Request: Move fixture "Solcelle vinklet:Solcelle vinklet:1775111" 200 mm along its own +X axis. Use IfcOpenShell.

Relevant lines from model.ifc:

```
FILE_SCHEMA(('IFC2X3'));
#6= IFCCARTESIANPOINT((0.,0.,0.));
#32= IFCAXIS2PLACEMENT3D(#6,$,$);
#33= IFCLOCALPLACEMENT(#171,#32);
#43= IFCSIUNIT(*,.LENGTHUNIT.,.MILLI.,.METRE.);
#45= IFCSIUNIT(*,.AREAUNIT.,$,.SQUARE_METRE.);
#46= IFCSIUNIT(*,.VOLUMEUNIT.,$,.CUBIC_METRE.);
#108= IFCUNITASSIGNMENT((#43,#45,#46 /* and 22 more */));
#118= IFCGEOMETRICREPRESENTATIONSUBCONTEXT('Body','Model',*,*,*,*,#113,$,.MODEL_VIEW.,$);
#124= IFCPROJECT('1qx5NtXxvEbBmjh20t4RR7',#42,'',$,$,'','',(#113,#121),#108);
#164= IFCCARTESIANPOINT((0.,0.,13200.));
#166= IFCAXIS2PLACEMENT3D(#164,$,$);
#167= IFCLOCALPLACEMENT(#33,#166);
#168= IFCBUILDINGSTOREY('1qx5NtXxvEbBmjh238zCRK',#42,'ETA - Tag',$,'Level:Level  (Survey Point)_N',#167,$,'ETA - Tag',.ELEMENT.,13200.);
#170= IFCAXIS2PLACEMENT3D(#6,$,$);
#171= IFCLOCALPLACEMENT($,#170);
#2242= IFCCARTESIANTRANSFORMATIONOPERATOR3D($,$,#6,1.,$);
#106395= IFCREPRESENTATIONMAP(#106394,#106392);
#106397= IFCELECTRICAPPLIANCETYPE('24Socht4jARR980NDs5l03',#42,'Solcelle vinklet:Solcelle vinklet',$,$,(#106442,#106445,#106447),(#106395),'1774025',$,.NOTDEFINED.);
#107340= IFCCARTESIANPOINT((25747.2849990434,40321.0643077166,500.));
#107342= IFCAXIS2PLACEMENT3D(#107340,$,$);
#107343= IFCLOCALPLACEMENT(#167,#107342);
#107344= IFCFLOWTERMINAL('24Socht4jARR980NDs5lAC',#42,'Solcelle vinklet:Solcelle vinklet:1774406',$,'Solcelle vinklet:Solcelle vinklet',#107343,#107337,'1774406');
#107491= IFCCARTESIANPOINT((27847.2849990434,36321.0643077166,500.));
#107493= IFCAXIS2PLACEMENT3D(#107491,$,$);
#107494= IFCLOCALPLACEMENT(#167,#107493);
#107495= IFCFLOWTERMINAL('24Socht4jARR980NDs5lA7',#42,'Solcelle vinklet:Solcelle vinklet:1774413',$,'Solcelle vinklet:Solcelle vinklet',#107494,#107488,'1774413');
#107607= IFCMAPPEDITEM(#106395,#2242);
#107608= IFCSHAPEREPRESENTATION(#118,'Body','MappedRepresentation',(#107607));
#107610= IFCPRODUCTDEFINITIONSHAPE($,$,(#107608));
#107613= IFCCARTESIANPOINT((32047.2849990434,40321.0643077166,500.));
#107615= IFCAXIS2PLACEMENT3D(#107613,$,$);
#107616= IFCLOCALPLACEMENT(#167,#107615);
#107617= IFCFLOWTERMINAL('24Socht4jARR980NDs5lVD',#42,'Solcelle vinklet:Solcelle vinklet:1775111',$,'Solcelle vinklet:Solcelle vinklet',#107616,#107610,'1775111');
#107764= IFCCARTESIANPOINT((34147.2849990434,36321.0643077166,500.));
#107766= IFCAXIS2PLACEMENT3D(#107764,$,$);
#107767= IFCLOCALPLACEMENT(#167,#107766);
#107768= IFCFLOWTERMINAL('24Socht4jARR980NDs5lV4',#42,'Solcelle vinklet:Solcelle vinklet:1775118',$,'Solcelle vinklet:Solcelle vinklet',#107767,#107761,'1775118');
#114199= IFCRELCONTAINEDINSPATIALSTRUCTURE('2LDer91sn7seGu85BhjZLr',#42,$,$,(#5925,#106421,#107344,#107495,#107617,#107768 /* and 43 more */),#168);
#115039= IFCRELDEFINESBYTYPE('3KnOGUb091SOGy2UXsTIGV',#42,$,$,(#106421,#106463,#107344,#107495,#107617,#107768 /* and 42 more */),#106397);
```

```python
import ifcopenshell
import ifcopenshell.api.geometry
import ifcopenshell.util.placement

model = ifcopenshell.open("model.ifc")

item = model.by_guid("24Socht4jARR980NDs5lVD")
matrix = ifcopenshell.util.placement.get_local_placement(item.ObjectPlacement)
matrix[:3, 3] += matrix[:3, 0] * 200.0
ifcopenshell.api.geometry.edit_object_placement(model, product=item, matrix=matrix, is_si=False)

print(ifcopenshell.util.placement.get_local_placement(item.ObjectPlacement).round(3) + 0.0)

model.write("model_rev.ifc")
```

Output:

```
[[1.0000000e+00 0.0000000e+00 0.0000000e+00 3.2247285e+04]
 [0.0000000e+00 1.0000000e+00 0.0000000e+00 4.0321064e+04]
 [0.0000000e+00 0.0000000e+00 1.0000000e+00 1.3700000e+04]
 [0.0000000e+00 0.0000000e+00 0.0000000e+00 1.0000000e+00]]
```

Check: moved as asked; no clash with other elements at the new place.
